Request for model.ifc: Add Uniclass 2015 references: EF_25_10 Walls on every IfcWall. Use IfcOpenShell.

First a look at what the model holds.

```python
import ifcopenshell

model = ifcopenshell.open("model.ifc")
print(model.schema)
print("classifications:", [c.Name for c in model.by_type("IfcClassification")])
for ifc_class in ("IfcDoor", "IfcRoof", "IfcStair", "IfcWall", "IfcWindow"):
    print(ifc_class, len(model.by_type(ifc_class)))
```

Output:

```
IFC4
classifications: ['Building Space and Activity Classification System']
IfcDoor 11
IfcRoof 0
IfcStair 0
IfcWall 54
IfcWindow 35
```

```python
import ifcopenshell
import ifcopenshell.api.classification

model = ifcopenshell.open("model.ifc")

system = ifcopenshell.api.classification.add_classification(model, classification="Uniclass 2015")

codes = {
    "IfcWall": ("EF_25_10", "Walls"),
}
for ifc_class, (code, name) in codes.items():
    products = model.by_type(ifc_class)
    ifcopenshell.api.classification.add_reference(
        model, products=products, classification=system, identification=code, name=name
    )
    print(code, len(products))

model.write("model_v2.ifc")
```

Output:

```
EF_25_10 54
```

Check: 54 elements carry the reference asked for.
